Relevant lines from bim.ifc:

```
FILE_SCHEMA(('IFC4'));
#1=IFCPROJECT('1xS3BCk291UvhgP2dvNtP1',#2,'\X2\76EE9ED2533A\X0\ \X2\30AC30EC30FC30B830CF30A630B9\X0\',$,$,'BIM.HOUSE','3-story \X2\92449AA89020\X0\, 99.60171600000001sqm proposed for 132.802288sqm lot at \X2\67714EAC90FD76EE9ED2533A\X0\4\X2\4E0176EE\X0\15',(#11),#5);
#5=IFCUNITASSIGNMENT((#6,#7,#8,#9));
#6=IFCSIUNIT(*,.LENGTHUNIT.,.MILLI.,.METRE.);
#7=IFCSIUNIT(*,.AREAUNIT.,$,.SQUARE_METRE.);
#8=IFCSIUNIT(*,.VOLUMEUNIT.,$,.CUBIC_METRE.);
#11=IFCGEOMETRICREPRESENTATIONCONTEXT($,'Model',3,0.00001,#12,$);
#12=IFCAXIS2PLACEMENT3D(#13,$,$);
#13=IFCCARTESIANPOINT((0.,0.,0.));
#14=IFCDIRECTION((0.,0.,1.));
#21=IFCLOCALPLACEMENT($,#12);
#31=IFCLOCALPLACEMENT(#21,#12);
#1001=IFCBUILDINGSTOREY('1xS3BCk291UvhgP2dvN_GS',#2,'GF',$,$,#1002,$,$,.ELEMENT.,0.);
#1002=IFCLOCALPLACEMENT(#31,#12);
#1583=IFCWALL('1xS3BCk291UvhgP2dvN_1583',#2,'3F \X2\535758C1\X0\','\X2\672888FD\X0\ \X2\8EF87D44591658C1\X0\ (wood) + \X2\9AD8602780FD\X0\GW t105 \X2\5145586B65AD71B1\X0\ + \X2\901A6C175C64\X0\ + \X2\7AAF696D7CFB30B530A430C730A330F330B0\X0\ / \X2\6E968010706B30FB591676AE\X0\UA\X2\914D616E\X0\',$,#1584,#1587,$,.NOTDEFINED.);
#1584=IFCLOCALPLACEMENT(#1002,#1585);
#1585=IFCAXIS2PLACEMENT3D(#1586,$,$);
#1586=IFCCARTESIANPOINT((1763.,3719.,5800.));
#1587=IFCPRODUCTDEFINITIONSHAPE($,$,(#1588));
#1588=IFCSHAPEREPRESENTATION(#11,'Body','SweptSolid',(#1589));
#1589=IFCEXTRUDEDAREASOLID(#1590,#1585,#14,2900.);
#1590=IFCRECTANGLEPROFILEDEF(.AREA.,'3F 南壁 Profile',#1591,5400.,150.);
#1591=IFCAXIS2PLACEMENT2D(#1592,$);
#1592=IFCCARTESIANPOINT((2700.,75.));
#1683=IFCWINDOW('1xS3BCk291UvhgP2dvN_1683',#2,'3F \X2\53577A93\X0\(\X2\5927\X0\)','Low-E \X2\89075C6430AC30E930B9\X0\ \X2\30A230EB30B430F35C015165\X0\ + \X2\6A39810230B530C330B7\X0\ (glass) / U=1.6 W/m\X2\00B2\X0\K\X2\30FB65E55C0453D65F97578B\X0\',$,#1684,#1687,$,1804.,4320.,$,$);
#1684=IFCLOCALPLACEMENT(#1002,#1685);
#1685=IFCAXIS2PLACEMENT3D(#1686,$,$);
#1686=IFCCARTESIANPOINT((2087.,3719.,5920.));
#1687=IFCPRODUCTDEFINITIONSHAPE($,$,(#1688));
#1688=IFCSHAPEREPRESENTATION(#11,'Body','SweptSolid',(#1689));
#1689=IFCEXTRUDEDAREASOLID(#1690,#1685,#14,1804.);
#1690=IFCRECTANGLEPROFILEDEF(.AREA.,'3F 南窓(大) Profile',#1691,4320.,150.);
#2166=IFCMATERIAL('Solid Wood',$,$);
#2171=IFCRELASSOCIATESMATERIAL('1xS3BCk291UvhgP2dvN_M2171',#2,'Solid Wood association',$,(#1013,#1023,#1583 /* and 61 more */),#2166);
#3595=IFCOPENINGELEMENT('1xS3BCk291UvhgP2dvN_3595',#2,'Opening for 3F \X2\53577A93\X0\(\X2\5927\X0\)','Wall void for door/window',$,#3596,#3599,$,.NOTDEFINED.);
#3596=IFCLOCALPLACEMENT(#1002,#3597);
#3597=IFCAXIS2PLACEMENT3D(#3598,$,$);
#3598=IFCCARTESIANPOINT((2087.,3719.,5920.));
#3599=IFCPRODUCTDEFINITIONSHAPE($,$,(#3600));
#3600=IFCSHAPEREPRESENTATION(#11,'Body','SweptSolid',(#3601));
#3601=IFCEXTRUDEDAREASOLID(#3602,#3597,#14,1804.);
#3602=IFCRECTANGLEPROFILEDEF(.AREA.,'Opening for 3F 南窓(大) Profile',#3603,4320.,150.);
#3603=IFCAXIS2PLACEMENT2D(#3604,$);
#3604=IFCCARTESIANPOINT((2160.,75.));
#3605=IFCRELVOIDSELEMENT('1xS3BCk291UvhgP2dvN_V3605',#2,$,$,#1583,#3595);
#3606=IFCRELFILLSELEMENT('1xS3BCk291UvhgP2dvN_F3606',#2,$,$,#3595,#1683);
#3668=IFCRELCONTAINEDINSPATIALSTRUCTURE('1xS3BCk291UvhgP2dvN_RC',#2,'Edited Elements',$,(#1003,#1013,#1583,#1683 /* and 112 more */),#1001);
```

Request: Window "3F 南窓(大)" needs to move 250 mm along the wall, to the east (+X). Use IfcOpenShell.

```python
import ifcopenshell
import ifcopenshell.api.geometry
import ifcopenshell.util.placement
import ifcopenshell.util.unit

model = ifcopenshell.open("bim.ifc")
unit_scale = ifcopenshell.util.unit.calculate_unit_scale(model)

window = model.by_guid("1xS3BCk291UvhgP2dvN_1683")
opening = window.FillsVoids[0].RelatingOpeningElement
wall = opening.VoidsElements[0].RelatingBuildingElement

wall_matrix = ifcopenshell.util.placement.get_local_placement(wall.ObjectPlacement)
shift = wall_matrix[:3, 0] * 0.25 / unit_scale
before = ifcopenshell.util.placement.get_local_placement(window.ObjectPlacement)[:3, 3].copy()

# The window is not placed relative to its opening, so move both.
for product in (opening, window):
    matrix = ifcopenshell.util.placement.get_local_placement(product.ObjectPlacement)
    matrix[:3, 3] += shift
    ifcopenshell.api.geometry.edit_object_placement(model, product=product, matrix=matrix, is_si=False)

after = ifcopenshell.util.placement.get_local_placement(window.ObjectPlacement)[:3, 3]
print("window moved by", (after - before).round(3) + 0.0)

model.write("bim_updated.ifc")
```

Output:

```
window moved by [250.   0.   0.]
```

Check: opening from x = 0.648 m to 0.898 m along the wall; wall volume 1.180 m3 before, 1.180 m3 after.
